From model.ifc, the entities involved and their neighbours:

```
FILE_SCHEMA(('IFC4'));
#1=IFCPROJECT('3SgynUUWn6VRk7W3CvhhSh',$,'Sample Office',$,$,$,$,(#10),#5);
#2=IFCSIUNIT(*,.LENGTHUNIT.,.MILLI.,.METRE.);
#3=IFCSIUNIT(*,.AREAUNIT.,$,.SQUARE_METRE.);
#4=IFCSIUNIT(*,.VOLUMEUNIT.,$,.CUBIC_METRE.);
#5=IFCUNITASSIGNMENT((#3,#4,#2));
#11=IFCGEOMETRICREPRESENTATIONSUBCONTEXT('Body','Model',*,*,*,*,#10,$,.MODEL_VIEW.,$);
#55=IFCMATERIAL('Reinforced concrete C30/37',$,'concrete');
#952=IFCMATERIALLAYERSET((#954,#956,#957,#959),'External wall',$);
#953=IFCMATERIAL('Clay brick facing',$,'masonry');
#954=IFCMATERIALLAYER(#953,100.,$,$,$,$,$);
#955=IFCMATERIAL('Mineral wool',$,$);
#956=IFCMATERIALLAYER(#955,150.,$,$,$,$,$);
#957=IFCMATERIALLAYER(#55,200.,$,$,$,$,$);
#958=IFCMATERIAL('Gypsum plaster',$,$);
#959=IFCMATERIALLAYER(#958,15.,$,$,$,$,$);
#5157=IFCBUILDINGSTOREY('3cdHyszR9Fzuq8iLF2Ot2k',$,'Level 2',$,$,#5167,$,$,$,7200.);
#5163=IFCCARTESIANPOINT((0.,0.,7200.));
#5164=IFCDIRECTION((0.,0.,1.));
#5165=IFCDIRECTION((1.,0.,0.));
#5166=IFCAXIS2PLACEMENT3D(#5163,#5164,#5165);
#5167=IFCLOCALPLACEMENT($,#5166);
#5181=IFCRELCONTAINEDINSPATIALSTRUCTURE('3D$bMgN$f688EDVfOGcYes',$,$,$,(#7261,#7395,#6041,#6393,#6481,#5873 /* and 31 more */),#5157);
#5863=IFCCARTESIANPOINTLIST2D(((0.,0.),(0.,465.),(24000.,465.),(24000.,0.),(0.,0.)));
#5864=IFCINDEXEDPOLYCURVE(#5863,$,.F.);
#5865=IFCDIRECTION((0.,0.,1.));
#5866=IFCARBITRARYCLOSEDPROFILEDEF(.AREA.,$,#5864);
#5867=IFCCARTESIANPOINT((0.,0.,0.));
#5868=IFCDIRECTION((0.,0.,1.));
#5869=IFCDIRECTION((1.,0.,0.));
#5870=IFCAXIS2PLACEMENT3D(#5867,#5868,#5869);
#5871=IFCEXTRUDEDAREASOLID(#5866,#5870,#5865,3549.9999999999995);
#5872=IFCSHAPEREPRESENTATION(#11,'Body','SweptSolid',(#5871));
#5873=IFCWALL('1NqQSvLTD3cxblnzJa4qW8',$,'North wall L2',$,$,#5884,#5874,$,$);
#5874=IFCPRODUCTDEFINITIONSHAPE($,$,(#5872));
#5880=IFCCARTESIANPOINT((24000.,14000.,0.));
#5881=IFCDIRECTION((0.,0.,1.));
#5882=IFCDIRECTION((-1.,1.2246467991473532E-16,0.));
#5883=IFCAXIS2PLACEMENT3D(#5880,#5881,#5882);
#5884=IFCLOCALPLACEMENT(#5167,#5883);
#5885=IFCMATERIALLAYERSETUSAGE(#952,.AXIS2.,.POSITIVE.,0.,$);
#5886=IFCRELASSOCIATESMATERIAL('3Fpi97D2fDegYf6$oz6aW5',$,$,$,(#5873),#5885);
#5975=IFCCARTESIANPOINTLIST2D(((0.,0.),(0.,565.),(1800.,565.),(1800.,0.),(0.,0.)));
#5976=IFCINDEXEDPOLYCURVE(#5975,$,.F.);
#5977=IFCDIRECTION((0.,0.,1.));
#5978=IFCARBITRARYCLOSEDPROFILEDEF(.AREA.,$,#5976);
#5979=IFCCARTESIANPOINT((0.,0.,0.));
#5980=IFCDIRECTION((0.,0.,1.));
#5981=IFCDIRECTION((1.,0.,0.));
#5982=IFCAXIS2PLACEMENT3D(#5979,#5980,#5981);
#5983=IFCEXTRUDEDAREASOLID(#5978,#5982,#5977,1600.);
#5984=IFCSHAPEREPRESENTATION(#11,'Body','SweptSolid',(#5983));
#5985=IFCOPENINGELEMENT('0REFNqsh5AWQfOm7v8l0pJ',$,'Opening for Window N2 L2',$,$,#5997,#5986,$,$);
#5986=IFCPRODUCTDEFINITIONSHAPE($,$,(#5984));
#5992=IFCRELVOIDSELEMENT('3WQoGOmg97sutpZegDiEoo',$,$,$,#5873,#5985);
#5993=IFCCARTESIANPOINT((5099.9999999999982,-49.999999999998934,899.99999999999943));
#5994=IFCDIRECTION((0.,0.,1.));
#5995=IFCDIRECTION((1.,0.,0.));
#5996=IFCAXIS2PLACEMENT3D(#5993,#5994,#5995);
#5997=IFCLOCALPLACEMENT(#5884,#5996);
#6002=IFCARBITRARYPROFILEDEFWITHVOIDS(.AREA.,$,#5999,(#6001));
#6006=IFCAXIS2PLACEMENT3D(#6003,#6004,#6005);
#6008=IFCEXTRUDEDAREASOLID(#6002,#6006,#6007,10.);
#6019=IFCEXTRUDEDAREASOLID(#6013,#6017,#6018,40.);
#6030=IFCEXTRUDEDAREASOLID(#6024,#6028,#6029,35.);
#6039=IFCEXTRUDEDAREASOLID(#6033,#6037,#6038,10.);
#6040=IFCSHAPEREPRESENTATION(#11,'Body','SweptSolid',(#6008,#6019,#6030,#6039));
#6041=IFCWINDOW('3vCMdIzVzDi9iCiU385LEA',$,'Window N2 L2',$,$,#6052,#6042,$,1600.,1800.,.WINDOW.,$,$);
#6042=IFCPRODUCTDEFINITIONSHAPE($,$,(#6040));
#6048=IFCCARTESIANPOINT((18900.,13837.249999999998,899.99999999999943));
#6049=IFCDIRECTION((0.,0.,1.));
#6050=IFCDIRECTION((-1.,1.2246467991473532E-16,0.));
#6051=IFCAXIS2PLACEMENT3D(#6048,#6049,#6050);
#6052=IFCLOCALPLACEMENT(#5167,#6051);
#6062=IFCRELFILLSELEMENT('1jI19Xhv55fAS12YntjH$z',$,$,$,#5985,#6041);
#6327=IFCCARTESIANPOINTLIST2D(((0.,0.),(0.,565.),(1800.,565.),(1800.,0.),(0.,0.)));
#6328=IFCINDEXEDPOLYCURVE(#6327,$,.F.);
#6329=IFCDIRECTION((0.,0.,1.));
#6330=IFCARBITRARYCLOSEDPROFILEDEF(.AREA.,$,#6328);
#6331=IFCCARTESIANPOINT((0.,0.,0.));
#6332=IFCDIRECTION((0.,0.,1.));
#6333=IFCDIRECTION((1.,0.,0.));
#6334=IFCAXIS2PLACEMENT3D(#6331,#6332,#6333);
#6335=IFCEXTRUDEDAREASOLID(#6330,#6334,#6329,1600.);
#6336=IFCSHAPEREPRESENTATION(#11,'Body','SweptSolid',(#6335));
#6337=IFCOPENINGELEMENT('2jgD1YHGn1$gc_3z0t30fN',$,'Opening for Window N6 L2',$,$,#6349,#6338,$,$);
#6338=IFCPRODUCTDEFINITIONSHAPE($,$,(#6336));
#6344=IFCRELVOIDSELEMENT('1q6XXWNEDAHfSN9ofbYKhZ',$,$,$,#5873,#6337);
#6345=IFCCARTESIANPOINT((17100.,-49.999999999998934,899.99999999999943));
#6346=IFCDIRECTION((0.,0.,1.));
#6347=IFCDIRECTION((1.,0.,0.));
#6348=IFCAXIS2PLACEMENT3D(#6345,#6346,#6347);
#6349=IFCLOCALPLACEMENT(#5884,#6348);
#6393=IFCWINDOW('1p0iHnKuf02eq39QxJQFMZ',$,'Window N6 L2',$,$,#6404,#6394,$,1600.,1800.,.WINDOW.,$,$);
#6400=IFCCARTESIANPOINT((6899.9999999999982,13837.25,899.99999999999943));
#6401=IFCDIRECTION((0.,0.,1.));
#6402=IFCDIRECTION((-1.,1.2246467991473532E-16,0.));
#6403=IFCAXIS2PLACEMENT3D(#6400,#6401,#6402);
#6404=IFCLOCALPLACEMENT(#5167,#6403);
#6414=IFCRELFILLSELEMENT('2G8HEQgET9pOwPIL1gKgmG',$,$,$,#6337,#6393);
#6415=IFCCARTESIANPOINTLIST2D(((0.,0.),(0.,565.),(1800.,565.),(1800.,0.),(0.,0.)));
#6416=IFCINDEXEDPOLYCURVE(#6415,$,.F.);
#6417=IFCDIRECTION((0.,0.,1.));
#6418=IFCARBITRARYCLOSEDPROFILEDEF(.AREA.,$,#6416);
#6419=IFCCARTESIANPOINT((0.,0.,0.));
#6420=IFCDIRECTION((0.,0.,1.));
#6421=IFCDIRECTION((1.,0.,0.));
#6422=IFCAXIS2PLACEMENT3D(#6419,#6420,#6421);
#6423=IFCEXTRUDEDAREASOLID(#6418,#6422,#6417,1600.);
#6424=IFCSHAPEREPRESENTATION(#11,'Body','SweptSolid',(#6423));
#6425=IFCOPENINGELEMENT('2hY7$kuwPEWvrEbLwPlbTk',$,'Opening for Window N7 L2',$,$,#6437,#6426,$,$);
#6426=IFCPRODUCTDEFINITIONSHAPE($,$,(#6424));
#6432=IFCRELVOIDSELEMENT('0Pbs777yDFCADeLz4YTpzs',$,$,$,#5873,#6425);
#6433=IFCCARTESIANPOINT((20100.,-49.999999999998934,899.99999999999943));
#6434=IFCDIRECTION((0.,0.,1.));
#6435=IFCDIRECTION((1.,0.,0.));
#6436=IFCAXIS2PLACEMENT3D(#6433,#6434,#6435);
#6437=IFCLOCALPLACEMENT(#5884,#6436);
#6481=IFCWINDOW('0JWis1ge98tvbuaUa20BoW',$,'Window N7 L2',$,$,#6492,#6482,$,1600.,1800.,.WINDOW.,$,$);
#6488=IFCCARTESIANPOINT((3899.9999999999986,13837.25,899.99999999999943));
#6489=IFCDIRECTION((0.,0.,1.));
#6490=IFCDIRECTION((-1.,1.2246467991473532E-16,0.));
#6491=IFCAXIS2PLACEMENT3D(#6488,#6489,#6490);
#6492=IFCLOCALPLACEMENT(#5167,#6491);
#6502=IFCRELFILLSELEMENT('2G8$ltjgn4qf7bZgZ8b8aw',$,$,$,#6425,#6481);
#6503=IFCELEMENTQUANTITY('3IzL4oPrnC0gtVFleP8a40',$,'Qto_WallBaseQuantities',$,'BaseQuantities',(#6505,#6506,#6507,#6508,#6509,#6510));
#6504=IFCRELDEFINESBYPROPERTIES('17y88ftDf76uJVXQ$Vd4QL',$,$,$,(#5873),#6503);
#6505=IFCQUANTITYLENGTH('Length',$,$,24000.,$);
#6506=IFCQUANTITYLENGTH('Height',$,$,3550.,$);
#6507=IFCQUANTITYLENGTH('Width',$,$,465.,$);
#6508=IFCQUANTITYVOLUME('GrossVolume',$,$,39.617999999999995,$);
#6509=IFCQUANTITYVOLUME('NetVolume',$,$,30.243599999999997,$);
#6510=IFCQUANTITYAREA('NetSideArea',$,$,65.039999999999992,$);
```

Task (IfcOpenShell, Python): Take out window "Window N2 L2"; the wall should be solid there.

```python
import ifcopenshell
import ifcopenshell.api.feature
import ifcopenshell.api.pset
import ifcopenshell.api.root
import ifcopenshell.geom
import ifcopenshell.util.element
import ifcopenshell.util.shape
import ifcopenshell.util.unit

model = ifcopenshell.open("model.ifc")
area_scale = ifcopenshell.util.unit.calculate_unit_scale(model, "AREAUNIT")
volume_scale = ifcopenshell.util.unit.calculate_unit_scale(model, "VOLUMEUNIT")
settings = ifcopenshell.geom.settings()


def volume(element):
    """Net volume in cubic metres, openings subtracted."""
    shape = ifcopenshell.geom.create_shape(settings, element)
    return ifcopenshell.util.shape.get_volume(shape.geometry)


window = model.by_guid("3vCMdIzVzDi9iCiU385LEA")
opening = window.FillsVoids[0].RelatingOpeningElement
wall = opening.VoidsElements[0].RelatingBuildingElement
before = volume(wall)

ifcopenshell.api.root.remove_product(model, product=window)
ifcopenshell.api.feature.remove_feature(model, feature=opening)

after = volume(wall)
thickness = 0.465  # wall thickness in metres

# Update the wall's stored quantities.
qto = model.by_id(ifcopenshell.util.element.get_pset(wall, "Qto_WallBaseQuantities", should_inherit=False)["id"])
ifcopenshell.api.pset.edit_qto(model, qto=qto, properties={
    "NetVolume": after / volume_scale,
    "NetSideArea": after / thickness / area_scale,
})

print(f"wall volume {before:.3f} -> {after:.3f} m3")

model.write("model-out.ifc")
```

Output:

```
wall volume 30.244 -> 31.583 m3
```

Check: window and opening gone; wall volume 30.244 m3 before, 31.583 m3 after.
